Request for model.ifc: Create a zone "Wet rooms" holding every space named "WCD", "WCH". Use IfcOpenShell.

First a look at what the model holds.

```python
import ifcopenshell

model = ifcopenshell.open("model.ifc")
print(model.schema)
seen = {}
for space in model.by_type("IfcSpace"):
    seen[space.LongName] = seen.get(space.LongName, 0) + 1
for name, count in sorted(seen.items(), key=str):
    print(count, "x", name)
print("zones:", [z.Name for z in model.by_type("IfcZone")][:20])
```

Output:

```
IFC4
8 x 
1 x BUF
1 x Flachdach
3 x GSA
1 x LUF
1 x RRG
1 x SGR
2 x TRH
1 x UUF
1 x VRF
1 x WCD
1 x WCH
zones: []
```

```python
import ifcopenshell
import ifcopenshell.api.group
import ifcopenshell.api.root

model = ifcopenshell.open("model.ifc")

names = {"WCD", "WCH"}
spaces = [s for s in model.by_type("IfcSpace") if s.LongName in names]

zone = ifcopenshell.api.root.create_entity(model, ifc_class="IfcZone", name="Wet rooms")
ifcopenshell.api.group.assign_group(model, products=spaces, group=zone)
print(len(spaces), "spaces in", zone.Name)

model.write("model_updated.ifc")
```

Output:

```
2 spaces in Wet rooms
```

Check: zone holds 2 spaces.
